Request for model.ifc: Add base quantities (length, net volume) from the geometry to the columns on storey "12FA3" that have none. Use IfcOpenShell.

First a look at what the model holds.

```python
import ifcopenshell
import ifcopenshell.util.element
import ifcopenshell.util.unit

model = ifcopenshell.open("model.ifc")
print(model.schema)
for unit_type in ("LENGTHUNIT", "AREAUNIT", "VOLUMEUNIT"):
    print(unit_type, ifcopenshell.util.unit.calculate_unit_scale(model, unit_type))
storey = next(s for s in model.by_type("IfcBuildingStorey") if s.Name == "12FA3")
columns = [e for e in ifcopenshell.util.element.get_decomposition(storey) if e.is_a("IfcColumn")]
for e in sorted(columns, key=lambda e: e.id()):
    print(e.id(), e.is_a(), e.Name, list(ifcopenshell.util.element.get_psets(e, qtos_only=True)), sep=" | ")
```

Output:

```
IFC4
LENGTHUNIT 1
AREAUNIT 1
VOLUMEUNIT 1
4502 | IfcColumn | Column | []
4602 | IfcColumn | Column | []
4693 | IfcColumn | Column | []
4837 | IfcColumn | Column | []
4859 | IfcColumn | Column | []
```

```python
import ifcopenshell
import ifcopenshell.api.pset
import ifcopenshell.geom
import ifcopenshell.util.element
import ifcopenshell.util.shape
import ifcopenshell.util.unit

model = ifcopenshell.open("model.ifc")
unit_scale = ifcopenshell.util.unit.calculate_unit_scale(model)
volume_scale = ifcopenshell.util.unit.calculate_unit_scale(model, "VOLUMEUNIT")
settings = ifcopenshell.geom.settings()

storey = next(s for s in model.by_type("IfcBuildingStorey") if s.Name == "12FA3")
columns = [e for e in ifcopenshell.util.element.get_decomposition(storey) if e.is_a("IfcColumn")]

for e in sorted(columns, key=lambda e: e.id()):
    if ifcopenshell.util.element.get_psets(e, qtos_only=True, should_inherit=False):
        continue
    # Geometry comes back in metres, in the element's own axes.
    shape = ifcopenshell.geom.create_shape(settings, e)
    values = {
        "Length": ifcopenshell.util.shape.get_z(shape.geometry) / unit_scale,
        "NetVolume": ifcopenshell.util.shape.get_volume(shape.geometry) / volume_scale,
    }
    qto = ifcopenshell.api.pset.add_qto(model, product=e, name="Qto_ColumnBaseQuantities")
    ifcopenshell.api.pset.edit_qto(model, qto=qto, properties=values)
    print(e.id(), {k: round(v, 3) for k, v in values.items()})

model.write("model-out.ifc")
```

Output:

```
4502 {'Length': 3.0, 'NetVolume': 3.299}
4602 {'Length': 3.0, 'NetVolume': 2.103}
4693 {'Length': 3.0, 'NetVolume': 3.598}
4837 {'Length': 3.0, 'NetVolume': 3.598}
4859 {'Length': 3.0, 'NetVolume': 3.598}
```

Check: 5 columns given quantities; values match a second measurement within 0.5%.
